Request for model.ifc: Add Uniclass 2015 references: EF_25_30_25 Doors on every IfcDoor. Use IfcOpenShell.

First a look at what the model holds.

```python
import ifcopenshell

model = ifcopenshell.open("model.ifc")
print(model.schema)
print("classifications:", [c.Name for c in model.by_type("IfcClassification")])
for ifc_class in ("IfcDoor", "IfcRoof", "IfcStair", "IfcWall", "IfcWindow"):
    print(ifc_class, len(model.by_type(ifc_class)))
```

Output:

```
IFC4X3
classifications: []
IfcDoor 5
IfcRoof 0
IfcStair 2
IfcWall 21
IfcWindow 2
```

```python
import ifcopenshell
import ifcopenshell.api.classification

model = ifcopenshell.open("model.ifc")

system = ifcopenshell.api.classification.add_classification(model, classification="Uniclass 2015")

codes = {
    "IfcDoor": ("EF_25_30_25", "Doors"),
}
for ifc_class, (code, name) in codes.items():
    products = model.by_type(ifc_class)
    ifcopenshell.api.classification.add_reference(
        model, products=products, classification=system, identification=code, name=name
    )
    print(code, len(products))

model.write("model_updated.ifc")
```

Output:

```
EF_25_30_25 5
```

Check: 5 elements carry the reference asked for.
